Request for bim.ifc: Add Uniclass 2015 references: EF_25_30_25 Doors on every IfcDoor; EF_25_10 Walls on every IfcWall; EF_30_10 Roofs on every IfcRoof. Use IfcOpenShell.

First a look at what the model holds.

```python
import ifcopenshell

model = ifcopenshell.open("bim.ifc")
print(model.schema)
print("classifications:", [c.Name for c in model.by_type("IfcClassification")])
for ifc_class in ("IfcDoor", "IfcRoof", "IfcStair", "IfcWall", "IfcWindow"):
    print(ifc_class, len(model.by_type(ifc_class)))
```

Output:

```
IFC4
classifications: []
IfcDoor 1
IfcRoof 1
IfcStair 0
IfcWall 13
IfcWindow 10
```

```python
import ifcopenshell
import ifcopenshell.api.classification

model = ifcopenshell.open("bim.ifc")

system = ifcopenshell.api.classification.add_classification(model, classification="Uniclass 2015")

codes = {
    "IfcDoor": ("EF_25_30_25", "Doors"),
    "IfcWall": ("EF_25_10", "Walls"),
    "IfcRoof": ("EF_30_10", "Roofs"),
}
for ifc_class, (code, name) in codes.items():
    products = model.by_type(ifc_class)
    ifcopenshell.api.classification.add_reference(
        model, products=products, classification=system, identification=code, name=name
    )
    print(code, len(products))

model.write("bim_rev.ifc")
```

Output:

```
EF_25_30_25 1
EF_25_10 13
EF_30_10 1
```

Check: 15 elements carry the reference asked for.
